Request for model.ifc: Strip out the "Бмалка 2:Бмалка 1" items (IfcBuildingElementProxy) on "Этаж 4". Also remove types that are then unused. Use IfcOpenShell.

First a look at what the model holds.

```python
import ifcopenshell
import ifcopenshell.util.element

model = ifcopenshell.open("model.ifc")
print(model.schema)
storey = next(s for s in model.by_type("IfcBuildingStorey") if s.Name == "Этаж 4")
proxies = [e for e in ifcopenshell.util.element.get_decomposition(storey) if e.is_a("IfcBuildingElementProxy")]
seen = {}
for e in proxies:
    element_type = ifcopenshell.util.element.get_type(e)
    name = element_type.Name if element_type not in (None, e) else None
    seen[name] = seen.get(name, 0) + 1
for name, count in sorted(seen.items(), key=str):
    print(count, "x", name)
```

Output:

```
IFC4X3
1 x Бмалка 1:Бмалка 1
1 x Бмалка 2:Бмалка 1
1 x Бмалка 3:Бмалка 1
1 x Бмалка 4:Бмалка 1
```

```python
import ifcopenshell
import ifcopenshell.api.root
import ifcopenshell.util.element

model = ifcopenshell.open("model.ifc")

storey = next(s for s in model.by_type("IfcBuildingStorey") if s.Name == "Этаж 4")
proxies = [e for e in ifcopenshell.util.element.get_decomposition(storey) if e.is_a("IfcBuildingElementProxy")]
targets = [e for e in proxies if (t := ifcopenshell.util.element.get_type(e)) not in (None, e) and t.Name == "Бмалка 2:Бмалка 1"]
types = {ifcopenshell.util.element.get_type(e) for e in targets} - {None, *targets}

for e in targets:
    ifcopenshell.api.root.remove_product(model, product=e)
print(len(targets), "removed")

unused = [t for t in types if not ifcopenshell.util.element.get_types(t)]
for t in unused:
    ifcopenshell.api.root.remove_product(model, product=t)
print(len(unused), "unused types removed")

model.write("model_edited.ifc")
```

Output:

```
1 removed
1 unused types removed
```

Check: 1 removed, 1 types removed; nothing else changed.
